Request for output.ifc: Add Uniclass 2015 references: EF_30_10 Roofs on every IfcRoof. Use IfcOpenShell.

First a look at what the model holds.

```python
import ifcopenshell

model = ifcopenshell.open("output.ifc")
print(model.schema)
print("classifications:", [c.Name for c in model.by_type("IfcClassification")])
for ifc_class in ("IfcDoor", "IfcRoof", "IfcStair", "IfcWall", "IfcWindow"):
    print(ifc_class, len(model.by_type(ifc_class)))
```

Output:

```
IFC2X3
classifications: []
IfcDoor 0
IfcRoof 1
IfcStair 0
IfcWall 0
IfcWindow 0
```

```python
import ifcopenshell
import ifcopenshell.api.classification

model = ifcopenshell.open("output.ifc")

# IFC2X3 requires Source and Edition and has no link from the project to the system.
system = model.create_entity("IfcClassification", Source="NBS", Edition="2015", Name="Uniclass 2015")

codes = {
    "IfcRoof": ("EF_30_10", "Roofs"),
}
for ifc_class, (code, name) in codes.items():
    products = model.by_type(ifc_class)
    ifcopenshell.api.classification.add_reference(
        model, products=products, classification=system, identification=code, name=name
    )
    print(code, len(products))

model.write("output_updated.ifc")
```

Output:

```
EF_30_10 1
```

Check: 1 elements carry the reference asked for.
